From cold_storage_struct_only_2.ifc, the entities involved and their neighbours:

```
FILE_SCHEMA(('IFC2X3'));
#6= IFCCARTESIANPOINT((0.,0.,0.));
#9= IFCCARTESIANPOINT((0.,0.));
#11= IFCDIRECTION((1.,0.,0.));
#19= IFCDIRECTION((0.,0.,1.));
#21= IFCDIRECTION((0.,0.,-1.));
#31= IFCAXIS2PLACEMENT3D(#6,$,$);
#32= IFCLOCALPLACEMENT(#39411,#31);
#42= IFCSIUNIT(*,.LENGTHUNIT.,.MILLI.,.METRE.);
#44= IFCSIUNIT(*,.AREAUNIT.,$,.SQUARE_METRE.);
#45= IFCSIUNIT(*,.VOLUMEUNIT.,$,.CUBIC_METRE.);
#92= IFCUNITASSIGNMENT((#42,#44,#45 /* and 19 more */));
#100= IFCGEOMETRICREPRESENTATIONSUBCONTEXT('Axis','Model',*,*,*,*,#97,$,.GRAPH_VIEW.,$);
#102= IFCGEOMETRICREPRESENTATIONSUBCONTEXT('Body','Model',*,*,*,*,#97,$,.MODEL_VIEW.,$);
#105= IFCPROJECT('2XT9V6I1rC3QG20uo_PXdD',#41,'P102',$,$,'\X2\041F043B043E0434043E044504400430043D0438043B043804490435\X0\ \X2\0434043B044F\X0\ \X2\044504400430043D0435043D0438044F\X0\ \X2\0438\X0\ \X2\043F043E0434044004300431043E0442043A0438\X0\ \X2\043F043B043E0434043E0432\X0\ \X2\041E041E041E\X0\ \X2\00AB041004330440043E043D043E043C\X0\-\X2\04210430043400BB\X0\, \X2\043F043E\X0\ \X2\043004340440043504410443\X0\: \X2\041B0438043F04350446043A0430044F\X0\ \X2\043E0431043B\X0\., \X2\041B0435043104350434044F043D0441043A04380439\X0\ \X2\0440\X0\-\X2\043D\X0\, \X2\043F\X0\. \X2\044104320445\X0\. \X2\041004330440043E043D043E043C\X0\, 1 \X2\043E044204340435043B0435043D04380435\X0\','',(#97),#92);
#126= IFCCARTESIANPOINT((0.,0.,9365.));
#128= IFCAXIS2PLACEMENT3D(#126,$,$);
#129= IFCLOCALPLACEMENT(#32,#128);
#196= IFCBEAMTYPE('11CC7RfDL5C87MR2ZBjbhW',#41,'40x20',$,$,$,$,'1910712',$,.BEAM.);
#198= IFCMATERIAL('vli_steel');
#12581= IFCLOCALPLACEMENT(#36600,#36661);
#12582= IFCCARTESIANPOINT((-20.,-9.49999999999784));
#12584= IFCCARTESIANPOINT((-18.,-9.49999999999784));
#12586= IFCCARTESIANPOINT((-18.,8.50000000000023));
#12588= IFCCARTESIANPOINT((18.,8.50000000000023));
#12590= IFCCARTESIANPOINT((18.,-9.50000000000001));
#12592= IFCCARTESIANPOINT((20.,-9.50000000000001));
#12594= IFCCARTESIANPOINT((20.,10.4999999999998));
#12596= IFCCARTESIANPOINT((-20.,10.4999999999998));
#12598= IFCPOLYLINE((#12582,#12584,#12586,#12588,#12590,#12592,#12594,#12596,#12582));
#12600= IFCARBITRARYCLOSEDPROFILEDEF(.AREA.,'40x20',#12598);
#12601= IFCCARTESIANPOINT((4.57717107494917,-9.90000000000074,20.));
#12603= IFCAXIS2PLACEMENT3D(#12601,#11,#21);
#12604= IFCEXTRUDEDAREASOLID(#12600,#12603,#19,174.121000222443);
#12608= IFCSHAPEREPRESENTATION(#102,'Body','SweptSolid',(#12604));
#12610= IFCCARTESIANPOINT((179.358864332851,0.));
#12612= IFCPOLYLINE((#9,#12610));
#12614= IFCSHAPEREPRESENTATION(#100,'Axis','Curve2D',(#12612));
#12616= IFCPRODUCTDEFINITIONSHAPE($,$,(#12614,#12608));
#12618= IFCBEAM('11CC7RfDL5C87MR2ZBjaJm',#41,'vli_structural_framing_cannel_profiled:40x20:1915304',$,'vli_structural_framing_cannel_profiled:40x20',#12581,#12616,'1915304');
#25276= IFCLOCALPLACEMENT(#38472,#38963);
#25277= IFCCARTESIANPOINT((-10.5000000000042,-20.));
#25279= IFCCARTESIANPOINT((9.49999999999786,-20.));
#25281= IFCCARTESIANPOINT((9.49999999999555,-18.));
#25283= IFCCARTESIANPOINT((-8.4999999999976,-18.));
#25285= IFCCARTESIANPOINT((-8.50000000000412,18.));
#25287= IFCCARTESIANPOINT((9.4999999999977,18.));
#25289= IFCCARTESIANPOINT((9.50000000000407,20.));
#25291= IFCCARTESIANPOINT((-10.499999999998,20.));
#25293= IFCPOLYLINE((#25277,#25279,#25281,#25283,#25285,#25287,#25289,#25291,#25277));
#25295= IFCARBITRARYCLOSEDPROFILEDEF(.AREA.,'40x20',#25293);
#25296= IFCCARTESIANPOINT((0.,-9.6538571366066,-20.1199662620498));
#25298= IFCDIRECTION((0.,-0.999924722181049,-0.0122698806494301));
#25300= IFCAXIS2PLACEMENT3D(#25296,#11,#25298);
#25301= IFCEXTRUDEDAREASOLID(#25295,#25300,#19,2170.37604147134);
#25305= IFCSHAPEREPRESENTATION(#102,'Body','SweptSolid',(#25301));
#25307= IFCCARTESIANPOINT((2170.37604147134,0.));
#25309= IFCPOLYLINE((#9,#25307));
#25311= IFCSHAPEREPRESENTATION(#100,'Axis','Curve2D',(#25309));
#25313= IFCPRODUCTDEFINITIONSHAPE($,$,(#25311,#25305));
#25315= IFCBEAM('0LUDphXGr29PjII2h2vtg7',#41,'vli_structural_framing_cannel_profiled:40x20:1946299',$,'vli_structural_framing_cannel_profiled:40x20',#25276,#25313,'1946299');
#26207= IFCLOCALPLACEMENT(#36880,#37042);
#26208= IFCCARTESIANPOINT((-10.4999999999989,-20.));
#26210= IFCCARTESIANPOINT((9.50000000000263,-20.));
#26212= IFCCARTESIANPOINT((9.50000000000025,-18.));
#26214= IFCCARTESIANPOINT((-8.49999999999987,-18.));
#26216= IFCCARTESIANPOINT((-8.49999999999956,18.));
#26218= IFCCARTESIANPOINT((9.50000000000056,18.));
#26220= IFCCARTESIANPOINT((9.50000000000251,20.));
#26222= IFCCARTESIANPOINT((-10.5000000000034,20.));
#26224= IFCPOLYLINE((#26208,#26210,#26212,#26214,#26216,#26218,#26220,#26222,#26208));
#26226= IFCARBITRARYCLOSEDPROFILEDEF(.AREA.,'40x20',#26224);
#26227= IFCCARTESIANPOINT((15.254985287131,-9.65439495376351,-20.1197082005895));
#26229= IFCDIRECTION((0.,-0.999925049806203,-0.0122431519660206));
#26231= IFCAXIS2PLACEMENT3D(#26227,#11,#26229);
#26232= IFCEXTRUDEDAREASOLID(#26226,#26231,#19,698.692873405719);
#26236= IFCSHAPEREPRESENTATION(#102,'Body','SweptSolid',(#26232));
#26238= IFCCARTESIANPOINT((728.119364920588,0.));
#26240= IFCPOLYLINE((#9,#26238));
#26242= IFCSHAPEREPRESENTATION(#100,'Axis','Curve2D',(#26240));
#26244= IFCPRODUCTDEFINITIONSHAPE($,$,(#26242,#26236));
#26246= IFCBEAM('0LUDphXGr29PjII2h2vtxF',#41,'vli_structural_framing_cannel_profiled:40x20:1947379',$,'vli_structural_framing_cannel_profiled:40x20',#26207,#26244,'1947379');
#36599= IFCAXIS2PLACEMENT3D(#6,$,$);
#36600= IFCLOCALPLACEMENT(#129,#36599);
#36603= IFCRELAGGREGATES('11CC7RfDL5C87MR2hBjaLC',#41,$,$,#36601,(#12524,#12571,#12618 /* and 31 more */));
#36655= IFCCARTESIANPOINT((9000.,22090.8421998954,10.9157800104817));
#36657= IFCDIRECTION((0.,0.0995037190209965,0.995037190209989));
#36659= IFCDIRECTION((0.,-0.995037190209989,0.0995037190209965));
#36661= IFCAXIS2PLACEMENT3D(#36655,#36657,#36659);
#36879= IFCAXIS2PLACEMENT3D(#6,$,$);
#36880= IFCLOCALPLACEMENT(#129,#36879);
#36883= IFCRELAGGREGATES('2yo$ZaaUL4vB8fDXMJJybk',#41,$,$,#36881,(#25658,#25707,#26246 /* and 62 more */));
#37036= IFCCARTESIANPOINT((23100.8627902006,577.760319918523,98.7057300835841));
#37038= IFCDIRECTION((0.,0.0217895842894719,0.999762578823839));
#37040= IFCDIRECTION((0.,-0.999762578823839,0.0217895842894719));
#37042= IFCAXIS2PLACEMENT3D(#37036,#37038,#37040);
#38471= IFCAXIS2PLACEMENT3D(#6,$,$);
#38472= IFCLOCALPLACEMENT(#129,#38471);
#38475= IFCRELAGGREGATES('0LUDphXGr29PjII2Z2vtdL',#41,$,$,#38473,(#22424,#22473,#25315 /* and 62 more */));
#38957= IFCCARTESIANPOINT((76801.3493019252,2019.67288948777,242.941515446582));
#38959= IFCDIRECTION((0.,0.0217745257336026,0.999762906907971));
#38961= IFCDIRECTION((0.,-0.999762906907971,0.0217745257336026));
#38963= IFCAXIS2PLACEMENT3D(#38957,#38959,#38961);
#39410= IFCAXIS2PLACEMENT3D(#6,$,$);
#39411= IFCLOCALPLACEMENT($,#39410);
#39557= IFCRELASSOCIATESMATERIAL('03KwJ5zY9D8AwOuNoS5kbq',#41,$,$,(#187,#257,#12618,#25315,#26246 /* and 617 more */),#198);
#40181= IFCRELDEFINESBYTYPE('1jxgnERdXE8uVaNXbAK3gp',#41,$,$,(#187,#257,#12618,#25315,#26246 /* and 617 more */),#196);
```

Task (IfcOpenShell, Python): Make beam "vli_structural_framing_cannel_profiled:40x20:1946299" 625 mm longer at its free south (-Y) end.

```python
import numpy as np
import ifcopenshell
import ifcopenshell.util.representation
import ifcopenshell.util.unit

model = ifcopenshell.open("cold_storage_struct_only_2.ifc")
unit_scale = ifcopenshell.util.unit.calculate_unit_scale(model)

member = model.by_id(25315)
change = 0.625 / unit_scale

# The extrusion runs towards the end named, so only its depth changes.
body = ifcopenshell.util.representation.get_representation(member, "Model", "Body")
solid = body.Items[0]
old_length = solid.Depth
solid.Depth += change

# Move the axis end point with it.
axis = next(r for r in member.Representation.Representations if r.RepresentationIdentifier == "Axis").Items[0]
start, end = (np.array(p.Coordinates) for p in axis.Points)
end = end + (end - start) / np.linalg.norm(end - start) * change
point = model.createIfcCartesianPoint(end.tolist())
axis.Points = [axis.Points[0], point]

print(f"length {old_length:g} -> {solid.Depth:g}")

model.write("cold_storage_struct_only_2_edited.ifc")
```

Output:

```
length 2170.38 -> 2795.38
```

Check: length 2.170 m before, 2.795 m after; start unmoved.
